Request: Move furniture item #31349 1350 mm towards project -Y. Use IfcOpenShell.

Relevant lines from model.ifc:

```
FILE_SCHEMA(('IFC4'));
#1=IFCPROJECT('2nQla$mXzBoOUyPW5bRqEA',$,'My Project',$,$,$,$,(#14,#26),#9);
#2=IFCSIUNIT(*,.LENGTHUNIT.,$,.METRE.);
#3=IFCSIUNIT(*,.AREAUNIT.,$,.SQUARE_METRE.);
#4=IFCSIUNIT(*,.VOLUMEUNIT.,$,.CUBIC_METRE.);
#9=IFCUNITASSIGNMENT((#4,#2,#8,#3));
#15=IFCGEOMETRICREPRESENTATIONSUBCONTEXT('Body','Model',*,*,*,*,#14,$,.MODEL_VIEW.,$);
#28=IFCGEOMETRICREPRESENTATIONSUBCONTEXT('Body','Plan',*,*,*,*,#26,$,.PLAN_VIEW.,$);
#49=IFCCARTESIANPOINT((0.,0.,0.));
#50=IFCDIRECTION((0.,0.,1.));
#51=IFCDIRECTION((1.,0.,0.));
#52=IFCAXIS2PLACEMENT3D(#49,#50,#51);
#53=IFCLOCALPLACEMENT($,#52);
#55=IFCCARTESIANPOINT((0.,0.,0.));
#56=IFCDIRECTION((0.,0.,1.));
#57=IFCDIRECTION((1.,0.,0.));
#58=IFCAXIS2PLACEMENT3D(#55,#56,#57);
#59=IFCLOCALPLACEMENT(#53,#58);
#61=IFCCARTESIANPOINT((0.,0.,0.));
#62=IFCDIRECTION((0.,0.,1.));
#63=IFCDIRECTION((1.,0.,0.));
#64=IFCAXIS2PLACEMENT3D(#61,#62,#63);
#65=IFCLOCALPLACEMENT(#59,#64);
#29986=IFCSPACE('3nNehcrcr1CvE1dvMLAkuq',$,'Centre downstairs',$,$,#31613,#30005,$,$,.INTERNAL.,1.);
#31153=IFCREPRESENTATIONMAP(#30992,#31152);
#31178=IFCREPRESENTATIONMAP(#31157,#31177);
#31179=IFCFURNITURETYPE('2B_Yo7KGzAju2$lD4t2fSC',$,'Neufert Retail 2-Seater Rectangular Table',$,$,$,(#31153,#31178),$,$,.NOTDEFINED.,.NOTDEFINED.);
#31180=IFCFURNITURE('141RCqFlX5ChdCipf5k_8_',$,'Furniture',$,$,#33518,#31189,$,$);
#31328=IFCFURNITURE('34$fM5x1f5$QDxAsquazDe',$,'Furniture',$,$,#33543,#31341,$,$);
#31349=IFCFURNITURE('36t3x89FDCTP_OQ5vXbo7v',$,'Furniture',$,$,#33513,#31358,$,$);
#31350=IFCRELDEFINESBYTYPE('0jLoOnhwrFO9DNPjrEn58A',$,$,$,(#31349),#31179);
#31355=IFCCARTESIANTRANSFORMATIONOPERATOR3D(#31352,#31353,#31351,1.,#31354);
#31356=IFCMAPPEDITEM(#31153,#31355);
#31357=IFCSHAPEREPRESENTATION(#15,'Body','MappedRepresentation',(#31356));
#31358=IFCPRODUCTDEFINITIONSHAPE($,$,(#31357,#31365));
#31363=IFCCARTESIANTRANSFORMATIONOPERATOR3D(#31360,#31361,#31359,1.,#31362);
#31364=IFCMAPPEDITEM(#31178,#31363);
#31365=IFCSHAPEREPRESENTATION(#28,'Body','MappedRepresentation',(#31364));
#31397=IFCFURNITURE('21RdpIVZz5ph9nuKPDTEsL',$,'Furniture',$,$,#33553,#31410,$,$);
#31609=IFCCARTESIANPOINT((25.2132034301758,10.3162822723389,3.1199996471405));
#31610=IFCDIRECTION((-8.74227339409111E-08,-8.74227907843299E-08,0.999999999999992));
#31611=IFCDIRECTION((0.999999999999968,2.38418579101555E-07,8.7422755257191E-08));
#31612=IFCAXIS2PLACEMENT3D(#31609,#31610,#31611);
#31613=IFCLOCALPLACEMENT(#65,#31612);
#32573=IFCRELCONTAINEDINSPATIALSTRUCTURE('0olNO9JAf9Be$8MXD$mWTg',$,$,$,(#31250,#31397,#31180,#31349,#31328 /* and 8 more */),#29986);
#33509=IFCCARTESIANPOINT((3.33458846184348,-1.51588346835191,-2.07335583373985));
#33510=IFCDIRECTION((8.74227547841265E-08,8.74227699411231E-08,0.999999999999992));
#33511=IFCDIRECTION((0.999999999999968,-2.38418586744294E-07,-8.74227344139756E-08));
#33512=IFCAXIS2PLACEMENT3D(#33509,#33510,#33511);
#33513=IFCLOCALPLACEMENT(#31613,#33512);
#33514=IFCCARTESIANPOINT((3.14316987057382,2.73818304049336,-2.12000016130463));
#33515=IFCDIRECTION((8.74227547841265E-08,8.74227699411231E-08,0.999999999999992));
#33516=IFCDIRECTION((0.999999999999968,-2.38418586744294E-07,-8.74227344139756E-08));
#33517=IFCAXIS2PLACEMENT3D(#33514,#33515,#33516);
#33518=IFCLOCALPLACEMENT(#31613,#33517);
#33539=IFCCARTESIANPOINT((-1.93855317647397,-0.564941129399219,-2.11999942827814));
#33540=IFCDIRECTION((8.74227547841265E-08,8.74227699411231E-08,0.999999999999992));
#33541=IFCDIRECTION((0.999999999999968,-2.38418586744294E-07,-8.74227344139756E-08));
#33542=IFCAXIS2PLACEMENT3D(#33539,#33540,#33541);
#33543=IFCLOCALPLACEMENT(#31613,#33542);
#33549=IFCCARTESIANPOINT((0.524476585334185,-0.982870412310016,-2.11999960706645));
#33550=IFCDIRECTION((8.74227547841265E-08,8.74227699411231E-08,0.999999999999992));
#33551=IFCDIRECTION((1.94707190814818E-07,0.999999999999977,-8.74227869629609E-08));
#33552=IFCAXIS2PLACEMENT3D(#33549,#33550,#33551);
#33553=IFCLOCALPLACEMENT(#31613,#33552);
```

```python
import ifcopenshell
import ifcopenshell.api.geometry
import ifcopenshell.util.placement
import ifcopenshell.util.unit

model = ifcopenshell.open("model.ifc")
unit_scale = ifcopenshell.util.unit.calculate_unit_scale(model)

item = model.by_guid("36t3x89FDCTP_OQ5vXbo7v")
matrix = ifcopenshell.util.placement.get_local_placement(item.ObjectPlacement)
matrix[1, 3] -= 1.35 / unit_scale
ifcopenshell.api.geometry.edit_object_placement(model, product=item, matrix=matrix, is_si=False)

print(ifcopenshell.util.placement.get_local_placement(item.ObjectPlacement).round(3) + 0.0)

model.write("model-out.ifc")
```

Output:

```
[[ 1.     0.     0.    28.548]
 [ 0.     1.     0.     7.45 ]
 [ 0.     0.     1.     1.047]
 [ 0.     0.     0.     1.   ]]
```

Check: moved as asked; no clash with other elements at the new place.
